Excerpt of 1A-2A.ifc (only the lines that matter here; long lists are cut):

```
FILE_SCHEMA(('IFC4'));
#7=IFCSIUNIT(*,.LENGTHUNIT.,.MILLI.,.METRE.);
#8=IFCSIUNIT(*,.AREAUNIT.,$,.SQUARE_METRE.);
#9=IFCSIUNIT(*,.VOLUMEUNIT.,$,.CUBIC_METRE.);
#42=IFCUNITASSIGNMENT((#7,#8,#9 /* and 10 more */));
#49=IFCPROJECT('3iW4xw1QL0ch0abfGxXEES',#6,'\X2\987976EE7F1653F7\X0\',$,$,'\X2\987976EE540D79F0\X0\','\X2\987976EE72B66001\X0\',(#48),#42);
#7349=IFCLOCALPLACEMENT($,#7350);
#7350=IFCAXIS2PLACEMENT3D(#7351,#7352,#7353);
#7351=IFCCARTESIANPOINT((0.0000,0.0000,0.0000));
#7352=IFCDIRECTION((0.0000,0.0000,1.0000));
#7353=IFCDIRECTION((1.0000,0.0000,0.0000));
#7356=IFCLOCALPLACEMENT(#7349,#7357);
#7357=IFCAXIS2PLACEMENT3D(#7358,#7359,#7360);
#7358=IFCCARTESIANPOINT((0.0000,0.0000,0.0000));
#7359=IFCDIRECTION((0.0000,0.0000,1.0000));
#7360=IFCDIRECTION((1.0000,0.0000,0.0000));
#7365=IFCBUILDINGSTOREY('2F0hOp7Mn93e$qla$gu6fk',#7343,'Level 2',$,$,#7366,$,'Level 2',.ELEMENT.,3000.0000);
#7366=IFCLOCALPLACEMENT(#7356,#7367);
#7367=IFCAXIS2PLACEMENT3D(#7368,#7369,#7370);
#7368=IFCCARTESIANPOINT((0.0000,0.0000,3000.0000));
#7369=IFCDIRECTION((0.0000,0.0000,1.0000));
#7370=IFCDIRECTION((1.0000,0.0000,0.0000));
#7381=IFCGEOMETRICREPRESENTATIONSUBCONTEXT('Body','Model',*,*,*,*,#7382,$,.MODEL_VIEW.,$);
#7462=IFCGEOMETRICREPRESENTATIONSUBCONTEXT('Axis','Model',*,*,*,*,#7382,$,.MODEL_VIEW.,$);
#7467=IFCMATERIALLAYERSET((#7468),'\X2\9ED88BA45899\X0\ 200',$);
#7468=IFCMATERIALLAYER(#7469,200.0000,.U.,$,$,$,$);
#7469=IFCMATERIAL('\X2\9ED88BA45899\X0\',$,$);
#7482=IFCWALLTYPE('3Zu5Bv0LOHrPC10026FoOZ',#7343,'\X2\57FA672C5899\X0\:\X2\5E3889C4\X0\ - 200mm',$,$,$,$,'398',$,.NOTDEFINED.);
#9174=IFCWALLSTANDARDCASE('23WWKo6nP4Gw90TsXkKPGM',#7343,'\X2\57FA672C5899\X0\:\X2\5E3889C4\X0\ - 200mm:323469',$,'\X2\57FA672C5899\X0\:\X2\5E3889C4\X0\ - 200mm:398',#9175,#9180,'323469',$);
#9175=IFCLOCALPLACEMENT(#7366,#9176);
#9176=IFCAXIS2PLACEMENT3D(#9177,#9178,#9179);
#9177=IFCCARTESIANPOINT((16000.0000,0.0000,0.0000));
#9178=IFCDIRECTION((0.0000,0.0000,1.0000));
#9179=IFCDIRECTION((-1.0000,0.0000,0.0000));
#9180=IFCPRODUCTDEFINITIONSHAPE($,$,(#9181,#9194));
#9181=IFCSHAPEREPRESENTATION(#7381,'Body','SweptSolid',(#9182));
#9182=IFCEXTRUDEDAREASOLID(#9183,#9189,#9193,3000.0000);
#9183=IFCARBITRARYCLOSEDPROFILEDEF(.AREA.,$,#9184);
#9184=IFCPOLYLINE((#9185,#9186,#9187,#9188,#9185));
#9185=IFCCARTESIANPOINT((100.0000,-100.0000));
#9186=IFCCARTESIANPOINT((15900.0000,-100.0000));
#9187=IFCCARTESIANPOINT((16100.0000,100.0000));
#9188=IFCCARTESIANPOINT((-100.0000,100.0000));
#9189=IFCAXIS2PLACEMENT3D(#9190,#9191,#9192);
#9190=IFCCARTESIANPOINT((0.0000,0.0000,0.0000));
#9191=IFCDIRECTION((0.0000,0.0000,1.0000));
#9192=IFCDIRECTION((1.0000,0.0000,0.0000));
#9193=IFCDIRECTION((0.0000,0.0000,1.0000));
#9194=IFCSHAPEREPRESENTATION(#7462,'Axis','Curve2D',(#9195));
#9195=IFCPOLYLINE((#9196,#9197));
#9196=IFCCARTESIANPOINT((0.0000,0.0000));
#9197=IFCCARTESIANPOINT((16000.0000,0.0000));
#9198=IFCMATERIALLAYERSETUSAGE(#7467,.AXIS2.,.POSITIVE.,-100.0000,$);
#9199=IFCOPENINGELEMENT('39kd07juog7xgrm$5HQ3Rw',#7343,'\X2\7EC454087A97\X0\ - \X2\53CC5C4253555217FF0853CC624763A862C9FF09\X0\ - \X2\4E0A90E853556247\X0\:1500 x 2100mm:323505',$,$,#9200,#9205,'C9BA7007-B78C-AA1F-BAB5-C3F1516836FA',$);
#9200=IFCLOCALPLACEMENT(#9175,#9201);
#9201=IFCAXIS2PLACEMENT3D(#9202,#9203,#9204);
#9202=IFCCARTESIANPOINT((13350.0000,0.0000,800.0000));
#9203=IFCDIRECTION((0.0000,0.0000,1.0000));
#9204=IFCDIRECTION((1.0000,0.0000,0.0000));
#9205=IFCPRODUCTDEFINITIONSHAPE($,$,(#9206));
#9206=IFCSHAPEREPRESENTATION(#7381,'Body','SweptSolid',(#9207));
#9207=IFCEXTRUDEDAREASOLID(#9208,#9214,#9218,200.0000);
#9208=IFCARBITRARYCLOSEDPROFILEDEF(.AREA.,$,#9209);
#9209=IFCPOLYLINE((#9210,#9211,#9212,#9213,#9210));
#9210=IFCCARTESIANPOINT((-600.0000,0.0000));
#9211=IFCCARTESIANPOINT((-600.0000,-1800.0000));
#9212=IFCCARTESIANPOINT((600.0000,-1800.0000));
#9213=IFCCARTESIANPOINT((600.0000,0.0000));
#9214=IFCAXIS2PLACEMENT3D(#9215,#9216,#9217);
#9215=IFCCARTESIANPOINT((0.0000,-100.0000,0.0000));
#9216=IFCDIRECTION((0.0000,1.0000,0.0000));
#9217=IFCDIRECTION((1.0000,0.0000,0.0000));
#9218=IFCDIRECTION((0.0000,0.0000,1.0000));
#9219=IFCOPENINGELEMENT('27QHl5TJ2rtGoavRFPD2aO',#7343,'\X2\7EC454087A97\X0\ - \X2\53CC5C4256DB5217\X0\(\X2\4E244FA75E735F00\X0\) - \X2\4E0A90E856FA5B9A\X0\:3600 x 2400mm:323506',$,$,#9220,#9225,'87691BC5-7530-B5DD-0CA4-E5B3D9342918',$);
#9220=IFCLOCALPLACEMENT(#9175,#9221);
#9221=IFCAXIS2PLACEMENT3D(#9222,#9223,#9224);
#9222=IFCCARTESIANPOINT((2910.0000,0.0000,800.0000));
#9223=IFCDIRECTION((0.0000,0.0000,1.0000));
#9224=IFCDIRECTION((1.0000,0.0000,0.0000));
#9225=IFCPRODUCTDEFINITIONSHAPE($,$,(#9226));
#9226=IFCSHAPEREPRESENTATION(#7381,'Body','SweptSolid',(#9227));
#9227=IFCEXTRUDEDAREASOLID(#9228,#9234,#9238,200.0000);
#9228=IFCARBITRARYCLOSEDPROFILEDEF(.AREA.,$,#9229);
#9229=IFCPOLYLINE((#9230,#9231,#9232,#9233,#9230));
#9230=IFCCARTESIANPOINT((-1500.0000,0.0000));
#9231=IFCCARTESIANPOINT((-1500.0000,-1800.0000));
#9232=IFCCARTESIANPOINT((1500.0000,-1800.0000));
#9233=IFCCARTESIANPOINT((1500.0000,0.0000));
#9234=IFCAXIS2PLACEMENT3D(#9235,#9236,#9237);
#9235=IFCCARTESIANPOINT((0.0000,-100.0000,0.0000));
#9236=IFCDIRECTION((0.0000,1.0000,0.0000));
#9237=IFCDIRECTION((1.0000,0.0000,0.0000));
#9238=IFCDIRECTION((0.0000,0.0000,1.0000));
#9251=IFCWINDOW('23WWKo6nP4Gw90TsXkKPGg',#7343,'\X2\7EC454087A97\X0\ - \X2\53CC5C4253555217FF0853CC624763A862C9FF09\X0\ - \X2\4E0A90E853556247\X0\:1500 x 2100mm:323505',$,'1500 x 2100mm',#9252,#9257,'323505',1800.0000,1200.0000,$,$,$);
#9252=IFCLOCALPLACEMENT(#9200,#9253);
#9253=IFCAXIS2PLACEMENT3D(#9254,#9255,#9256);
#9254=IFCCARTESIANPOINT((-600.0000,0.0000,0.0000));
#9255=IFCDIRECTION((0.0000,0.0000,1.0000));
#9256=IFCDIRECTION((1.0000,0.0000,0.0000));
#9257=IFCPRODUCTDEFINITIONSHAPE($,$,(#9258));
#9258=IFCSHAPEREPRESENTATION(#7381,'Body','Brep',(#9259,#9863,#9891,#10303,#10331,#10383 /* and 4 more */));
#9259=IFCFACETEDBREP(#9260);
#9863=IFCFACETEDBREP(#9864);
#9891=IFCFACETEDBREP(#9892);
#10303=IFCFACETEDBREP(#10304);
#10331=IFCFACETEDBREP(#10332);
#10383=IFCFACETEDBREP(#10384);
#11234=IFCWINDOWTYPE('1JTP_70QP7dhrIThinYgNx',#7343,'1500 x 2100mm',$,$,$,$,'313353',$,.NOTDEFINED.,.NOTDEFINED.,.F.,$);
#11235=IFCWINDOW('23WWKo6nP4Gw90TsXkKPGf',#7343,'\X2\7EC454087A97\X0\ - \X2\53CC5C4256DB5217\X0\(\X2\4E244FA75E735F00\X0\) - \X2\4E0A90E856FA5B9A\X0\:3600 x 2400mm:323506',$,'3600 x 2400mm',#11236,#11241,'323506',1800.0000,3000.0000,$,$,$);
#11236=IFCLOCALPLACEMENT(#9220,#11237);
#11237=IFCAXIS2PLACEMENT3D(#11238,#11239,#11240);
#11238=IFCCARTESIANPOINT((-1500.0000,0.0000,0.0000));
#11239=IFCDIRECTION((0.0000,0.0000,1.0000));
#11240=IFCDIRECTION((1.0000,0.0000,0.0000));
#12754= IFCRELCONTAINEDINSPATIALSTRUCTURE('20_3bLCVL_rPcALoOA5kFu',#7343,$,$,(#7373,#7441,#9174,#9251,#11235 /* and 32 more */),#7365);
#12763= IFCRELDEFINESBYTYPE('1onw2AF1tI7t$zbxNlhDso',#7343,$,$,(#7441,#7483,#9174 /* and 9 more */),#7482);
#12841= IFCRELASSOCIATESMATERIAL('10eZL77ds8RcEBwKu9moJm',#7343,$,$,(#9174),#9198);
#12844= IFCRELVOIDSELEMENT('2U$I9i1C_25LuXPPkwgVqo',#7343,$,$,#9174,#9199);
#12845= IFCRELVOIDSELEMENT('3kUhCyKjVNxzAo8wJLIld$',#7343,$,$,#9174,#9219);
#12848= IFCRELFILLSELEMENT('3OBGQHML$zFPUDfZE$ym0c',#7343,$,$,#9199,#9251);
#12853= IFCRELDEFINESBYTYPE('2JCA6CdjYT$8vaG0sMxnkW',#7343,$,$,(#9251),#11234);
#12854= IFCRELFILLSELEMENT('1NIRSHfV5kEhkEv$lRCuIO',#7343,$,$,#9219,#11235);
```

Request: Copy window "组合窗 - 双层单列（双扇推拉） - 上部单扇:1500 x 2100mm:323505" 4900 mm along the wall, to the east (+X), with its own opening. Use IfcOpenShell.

```python
import ifcopenshell
import ifcopenshell.api.feature
import ifcopenshell.api.geometry
import ifcopenshell.api.root
import ifcopenshell.geom
import ifcopenshell.util.element
import ifcopenshell.util.placement
import ifcopenshell.util.shape
import ifcopenshell.util.unit

model = ifcopenshell.open("1A-2A.ifc")
unit_scale = ifcopenshell.util.unit.calculate_unit_scale(model)
settings = ifcopenshell.geom.settings()


def volume(element):
    """Net volume in cubic metres, openings subtracted."""
    shape = ifcopenshell.geom.create_shape(settings, element)
    return ifcopenshell.util.shape.get_volume(shape.geometry)


def reuse_history(source, copy):
    """copy_class also copies each property set's owner history, people and application; keep the originals."""
    for rel in copy.IsDefinedBy:
        if rel.is_a("IfcRelDefinesByProperties") and (history := rel.RelatingPropertyDefinition.OwnerHistory):
            rel.RelatingPropertyDefinition.OwnerHistory = source.OwnerHistory
            ifcopenshell.util.element.remove_deep2(model, history)


window = model.by_id(9251)
opening = window.FillsVoids[0].RelatingOpeningElement
wall = opening.VoidsElements[0].RelatingBuildingElement
before = volume(wall)
shift = ifcopenshell.util.placement.get_local_placement(wall.ObjectPlacement)[:3, 0] * -4.9 / unit_scale

# copy_class copies the void relationship, type, container and properties, but no geometry.
new_opening = ifcopenshell.api.root.copy_class(model, product=opening)
new_opening.Representation = ifcopenshell.util.element.copy_deep(
    model, opening.Representation, exclude=["IfcGeometricRepresentationContext", "IfcRepresentationMap"]
)
new_opening.Name = "组合窗 - 双层单列（双扇推拉） - 上部单扇:1500 x 2100mm"
new_opening.Tag = None
new_window = ifcopenshell.api.root.copy_class(model, product=window)
new_window.Representation = ifcopenshell.util.element.copy_deep(
    model, window.Representation, exclude=["IfcGeometricRepresentationContext", "IfcRepresentationMap"]
)
new_window.Name = "组合窗 - 双层单列（双扇推拉） - 上部单扇:1500 x 2100mm"
new_window.Tag = None
reuse_history(window, new_window)
ifcopenshell.api.feature.add_filling(model, opening=new_opening, element=new_window)

for old, new in ((opening, new_opening), (window, new_window)):
    matrix = ifcopenshell.util.placement.get_local_placement(old.ObjectPlacement)
    matrix[:3, 3] += shift
    ifcopenshell.api.geometry.edit_object_placement(model, product=new, matrix=matrix, is_si=False)

after = volume(wall)

print(f"wall volume {before:.3f} -> {after:.3f} m3")

model.write("1A-2A_updated.ifc")
```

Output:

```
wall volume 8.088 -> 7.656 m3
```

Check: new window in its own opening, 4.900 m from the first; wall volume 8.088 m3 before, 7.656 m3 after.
